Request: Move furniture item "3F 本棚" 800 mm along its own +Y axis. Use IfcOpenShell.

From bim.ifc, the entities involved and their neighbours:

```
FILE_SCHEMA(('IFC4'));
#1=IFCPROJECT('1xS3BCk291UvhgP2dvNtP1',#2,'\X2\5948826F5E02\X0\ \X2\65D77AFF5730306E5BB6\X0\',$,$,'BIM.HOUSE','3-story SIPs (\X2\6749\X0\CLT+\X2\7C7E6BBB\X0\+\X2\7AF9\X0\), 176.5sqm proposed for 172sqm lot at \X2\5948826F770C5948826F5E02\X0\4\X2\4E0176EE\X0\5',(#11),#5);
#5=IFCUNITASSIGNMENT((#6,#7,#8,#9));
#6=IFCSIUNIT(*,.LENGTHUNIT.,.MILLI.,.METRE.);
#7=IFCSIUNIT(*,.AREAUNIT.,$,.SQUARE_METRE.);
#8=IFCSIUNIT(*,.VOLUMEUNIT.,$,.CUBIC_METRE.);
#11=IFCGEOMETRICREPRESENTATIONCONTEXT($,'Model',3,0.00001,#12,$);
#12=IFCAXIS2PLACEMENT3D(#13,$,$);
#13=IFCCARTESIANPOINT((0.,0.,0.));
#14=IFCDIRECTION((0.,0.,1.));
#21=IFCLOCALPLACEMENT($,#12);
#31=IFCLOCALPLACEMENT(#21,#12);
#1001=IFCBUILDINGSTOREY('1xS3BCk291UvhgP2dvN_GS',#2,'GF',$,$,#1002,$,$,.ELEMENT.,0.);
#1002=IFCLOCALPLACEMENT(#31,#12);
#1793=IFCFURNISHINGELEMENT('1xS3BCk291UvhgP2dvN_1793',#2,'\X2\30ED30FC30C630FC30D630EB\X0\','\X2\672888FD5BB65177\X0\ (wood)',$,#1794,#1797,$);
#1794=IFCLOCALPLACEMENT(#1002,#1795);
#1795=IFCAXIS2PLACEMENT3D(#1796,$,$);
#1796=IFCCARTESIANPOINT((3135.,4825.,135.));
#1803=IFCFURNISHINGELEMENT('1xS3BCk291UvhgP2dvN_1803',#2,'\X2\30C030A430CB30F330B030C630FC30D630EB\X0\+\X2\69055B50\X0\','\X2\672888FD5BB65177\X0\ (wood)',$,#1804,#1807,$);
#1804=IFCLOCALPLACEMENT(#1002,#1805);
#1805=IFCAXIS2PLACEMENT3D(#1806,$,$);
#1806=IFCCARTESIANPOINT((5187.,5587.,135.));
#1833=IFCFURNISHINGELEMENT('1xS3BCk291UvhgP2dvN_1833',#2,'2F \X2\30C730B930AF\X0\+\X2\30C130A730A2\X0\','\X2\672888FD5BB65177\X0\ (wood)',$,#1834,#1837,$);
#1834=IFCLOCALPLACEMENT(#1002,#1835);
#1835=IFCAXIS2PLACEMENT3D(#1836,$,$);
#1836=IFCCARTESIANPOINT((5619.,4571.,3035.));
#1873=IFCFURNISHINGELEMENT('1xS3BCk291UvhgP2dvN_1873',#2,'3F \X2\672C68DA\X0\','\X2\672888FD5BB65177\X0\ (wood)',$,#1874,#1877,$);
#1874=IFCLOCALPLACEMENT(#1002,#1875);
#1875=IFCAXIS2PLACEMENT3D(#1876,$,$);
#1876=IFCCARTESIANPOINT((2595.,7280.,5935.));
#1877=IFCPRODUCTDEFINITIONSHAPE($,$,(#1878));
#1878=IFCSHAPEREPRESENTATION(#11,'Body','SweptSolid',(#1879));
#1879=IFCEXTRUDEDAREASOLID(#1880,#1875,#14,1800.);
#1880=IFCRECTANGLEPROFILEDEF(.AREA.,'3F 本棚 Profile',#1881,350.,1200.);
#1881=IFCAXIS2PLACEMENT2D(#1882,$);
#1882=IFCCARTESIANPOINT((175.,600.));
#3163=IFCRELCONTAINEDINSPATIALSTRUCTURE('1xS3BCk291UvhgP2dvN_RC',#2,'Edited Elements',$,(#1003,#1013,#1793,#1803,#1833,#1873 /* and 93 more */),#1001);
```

```python
import ifcopenshell
import ifcopenshell.api.geometry
import ifcopenshell.util.placement

model = ifcopenshell.open("bim.ifc")

item = model.by_guid("1xS3BCk291UvhgP2dvN_1873")
matrix = ifcopenshell.util.placement.get_local_placement(item.ObjectPlacement)
matrix[:3, 3] += matrix[:3, 1] * 800.0
ifcopenshell.api.geometry.edit_object_placement(model, product=item, matrix=matrix, is_si=False)

print(ifcopenshell.util.placement.get_local_placement(item.ObjectPlacement).round(3) + 0.0)

model.write("bim_edited.ifc")
```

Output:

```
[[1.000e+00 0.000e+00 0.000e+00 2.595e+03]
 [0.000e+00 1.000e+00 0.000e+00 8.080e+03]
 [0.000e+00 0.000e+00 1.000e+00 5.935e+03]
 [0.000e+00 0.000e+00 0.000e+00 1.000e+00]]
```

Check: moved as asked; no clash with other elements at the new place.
